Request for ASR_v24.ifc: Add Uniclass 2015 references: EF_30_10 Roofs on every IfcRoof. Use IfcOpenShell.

First a look at what the model holds.

```python
import ifcopenshell

model = ifcopenshell.open("ASR_v24.ifc")
print(model.schema)
print("classifications:", [c.Name for c in model.by_type("IfcClassification")])
for ifc_class in ("IfcDoor", "IfcRoof", "IfcStair", "IfcWall", "IfcWindow"):
    print(ifc_class, len(model.by_type(ifc_class)))
```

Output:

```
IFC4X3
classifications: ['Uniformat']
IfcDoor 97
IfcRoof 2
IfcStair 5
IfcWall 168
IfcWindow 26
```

```python
import ifcopenshell
import ifcopenshell.api.classification

model = ifcopenshell.open("ASR_v24.ifc")

system = ifcopenshell.api.classification.add_classification(model, classification="Uniclass 2015")

codes = {
    "IfcRoof": ("EF_30_10", "Roofs"),
}
for ifc_class, (code, name) in codes.items():
    products = model.by_type(ifc_class)
    ifcopenshell.api.classification.add_reference(
        model, products=products, classification=system, identification=code, name=name
    )
    print(code, len(products))

model.write("ASR_v24_edited.ifc")
```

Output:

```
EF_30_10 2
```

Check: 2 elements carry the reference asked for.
